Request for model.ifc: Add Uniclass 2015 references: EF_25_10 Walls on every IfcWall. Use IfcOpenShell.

First a look at what the model holds.

```python
import ifcopenshell

model = ifcopenshell.open("model.ifc")
print(model.schema)
print("classifications:", [c.Name for c in model.by_type("IfcClassification")])
for ifc_class in ("IfcDoor", "IfcRoof", "IfcStair", "IfcWall", "IfcWindow"):
    print(ifc_class, len(model.by_type(ifc_class)))
```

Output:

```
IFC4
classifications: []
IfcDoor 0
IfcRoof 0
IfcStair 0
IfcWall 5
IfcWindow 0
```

```python
import ifcopenshell
import ifcopenshell.api.classification

model = ifcopenshell.open("model.ifc")

system = ifcopenshell.api.classification.add_classification(model, classification="Uniclass 2015")

codes = {
    "IfcWall": ("EF_25_10", "Walls"),
}
for ifc_class, (code, name) in codes.items():
    products = model.by_type(ifc_class)
    ifcopenshell.api.classification.add_reference(
        model, products=products, classification=system, identification=code, name=name
    )
    print(code, len(products))

model.write("model_edited.ifc")
```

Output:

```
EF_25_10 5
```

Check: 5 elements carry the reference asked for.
